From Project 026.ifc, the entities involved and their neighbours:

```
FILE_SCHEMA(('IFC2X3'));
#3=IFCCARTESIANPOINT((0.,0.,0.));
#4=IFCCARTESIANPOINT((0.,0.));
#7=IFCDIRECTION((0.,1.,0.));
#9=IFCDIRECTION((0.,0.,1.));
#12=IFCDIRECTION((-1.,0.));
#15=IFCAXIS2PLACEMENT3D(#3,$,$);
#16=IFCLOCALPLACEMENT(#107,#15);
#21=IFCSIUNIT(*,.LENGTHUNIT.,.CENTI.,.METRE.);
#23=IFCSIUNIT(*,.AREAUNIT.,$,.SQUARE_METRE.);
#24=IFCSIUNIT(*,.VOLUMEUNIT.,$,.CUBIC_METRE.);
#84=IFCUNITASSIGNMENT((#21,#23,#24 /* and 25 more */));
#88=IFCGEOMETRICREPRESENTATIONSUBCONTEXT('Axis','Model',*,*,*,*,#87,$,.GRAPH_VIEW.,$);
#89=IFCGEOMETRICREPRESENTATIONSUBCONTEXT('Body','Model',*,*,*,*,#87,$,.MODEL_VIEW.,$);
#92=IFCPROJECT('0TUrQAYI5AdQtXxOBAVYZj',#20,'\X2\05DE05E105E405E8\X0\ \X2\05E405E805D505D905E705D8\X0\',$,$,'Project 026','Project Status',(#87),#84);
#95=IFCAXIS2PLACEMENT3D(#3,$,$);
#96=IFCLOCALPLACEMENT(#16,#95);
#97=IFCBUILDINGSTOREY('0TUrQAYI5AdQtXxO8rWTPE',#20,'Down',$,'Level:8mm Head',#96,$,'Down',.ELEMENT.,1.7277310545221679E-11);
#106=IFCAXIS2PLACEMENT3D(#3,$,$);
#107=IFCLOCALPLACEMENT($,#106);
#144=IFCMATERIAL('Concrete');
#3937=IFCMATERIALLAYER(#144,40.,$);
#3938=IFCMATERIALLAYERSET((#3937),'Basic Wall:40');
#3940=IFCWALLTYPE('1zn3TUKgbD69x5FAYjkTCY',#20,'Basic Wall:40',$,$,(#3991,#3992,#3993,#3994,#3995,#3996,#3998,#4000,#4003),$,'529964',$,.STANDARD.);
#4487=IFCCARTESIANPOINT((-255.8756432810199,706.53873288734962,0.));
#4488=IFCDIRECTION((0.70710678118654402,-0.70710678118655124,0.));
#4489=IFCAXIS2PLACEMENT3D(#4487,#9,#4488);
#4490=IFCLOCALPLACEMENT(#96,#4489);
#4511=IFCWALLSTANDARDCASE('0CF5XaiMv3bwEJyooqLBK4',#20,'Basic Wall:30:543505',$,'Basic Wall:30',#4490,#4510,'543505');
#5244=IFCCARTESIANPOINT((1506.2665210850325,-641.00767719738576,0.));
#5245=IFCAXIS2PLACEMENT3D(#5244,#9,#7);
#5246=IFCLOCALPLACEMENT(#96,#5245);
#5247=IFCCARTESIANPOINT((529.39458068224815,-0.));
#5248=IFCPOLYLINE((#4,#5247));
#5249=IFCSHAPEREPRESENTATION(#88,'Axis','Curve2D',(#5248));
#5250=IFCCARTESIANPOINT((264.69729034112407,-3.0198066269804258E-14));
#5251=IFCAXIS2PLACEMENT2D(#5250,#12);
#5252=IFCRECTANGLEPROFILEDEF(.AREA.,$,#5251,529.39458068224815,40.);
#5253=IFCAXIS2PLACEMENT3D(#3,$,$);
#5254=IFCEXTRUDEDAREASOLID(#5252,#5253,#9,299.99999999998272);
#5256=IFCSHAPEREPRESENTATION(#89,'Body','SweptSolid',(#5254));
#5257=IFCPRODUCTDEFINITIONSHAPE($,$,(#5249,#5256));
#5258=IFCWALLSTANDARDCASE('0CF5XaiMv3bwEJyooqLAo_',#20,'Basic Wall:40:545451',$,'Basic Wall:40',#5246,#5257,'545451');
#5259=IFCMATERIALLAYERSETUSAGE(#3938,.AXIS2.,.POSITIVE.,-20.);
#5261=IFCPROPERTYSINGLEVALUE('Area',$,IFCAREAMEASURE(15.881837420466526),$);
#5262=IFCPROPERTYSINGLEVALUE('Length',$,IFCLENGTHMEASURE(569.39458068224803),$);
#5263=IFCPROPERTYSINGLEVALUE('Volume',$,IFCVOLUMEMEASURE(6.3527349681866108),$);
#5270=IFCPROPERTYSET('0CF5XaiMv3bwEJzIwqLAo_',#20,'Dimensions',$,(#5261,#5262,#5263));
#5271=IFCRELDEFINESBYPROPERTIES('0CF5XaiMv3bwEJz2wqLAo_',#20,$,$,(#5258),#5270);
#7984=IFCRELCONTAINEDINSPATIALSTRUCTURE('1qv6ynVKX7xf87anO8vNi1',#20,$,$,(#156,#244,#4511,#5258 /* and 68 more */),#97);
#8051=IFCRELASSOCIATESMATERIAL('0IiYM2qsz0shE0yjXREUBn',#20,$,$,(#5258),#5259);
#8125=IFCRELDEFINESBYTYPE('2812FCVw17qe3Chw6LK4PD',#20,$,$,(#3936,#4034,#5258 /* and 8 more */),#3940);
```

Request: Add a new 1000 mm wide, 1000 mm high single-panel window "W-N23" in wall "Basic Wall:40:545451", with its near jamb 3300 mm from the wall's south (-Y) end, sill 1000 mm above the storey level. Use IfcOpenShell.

```python
import numpy as np
import ifcopenshell
import ifcopenshell.api.feature
import ifcopenshell.api.geometry
import ifcopenshell.api.pset
import ifcopenshell.api.root
import ifcopenshell.api.spatial
import ifcopenshell.api.type
import ifcopenshell.geom
import ifcopenshell.util.element
import ifcopenshell.util.placement
import ifcopenshell.util.representation
import ifcopenshell.util.shape
import ifcopenshell.util.unit

model = ifcopenshell.open("Project 026.ifc")
unit_scale = ifcopenshell.util.unit.calculate_unit_scale(model)
area_scale = ifcopenshell.util.unit.calculate_unit_scale(model, "AREAUNIT")
volume_scale = ifcopenshell.util.unit.calculate_unit_scale(model, "VOLUMEUNIT")
settings = ifcopenshell.geom.settings()


def volume(element):
    """Net volume in cubic metres, openings subtracted."""
    shape = ifcopenshell.geom.create_shape(settings, element)
    return ifcopenshell.util.shape.get_volume(shape.geometry)


wall = model.by_guid("0CF5XaiMv3bwEJyooqLAo_")
storey = ifcopenshell.util.element.get_container(wall, ifc_class="IfcBuildingStorey")
context = ifcopenshell.util.representation.get_context(model, "Model", "Body", "MODEL_VIEW")
before = volume(wall)

width, height, from_end, sill = 1, 1, 3.3, 1  # metres

# The wall runs along its own X axis, and the end named is its -X end.
wall_shape = ifcopenshell.geom.create_shape(settings, wall)
x, y, z = ifcopenshell.util.shape.get_vertices(wall_shape.geometry).T
start = x.min() + from_end
face, thickness = float(y.min()), float(y.max() - y.min())
wall_matrix = ifcopenshell.util.placement.get_local_placement(wall.ObjectPlacement)
level = ifcopenshell.util.placement.get_local_placement(storey.ObjectPlacement)[2, 3]


def in_wall(x, y):
    """Placement at x, y metres in the wall's axes, at sill height."""
    matrix = wall_matrix.copy()
    matrix[:, 3] = wall_matrix @ np.array([x / unit_scale, y / unit_scale, 0.0, 1.0])
    matrix[2, 3] = level + sill / unit_scale
    return matrix


# Opening: a box that overshoots both wall faces by 50 mm.
opening = ifcopenshell.api.root.create_entity(model, ifc_class="IfcOpeningElement")
box = ifcopenshell.api.geometry.add_wall_representation(
    model, context=context, length=width, height=height, thickness=thickness + 0.1
)
ifcopenshell.api.geometry.assign_representation(model, product=opening, representation=box)
ifcopenshell.api.geometry.edit_object_placement(model, product=opening, matrix=in_wall(start, face - 0.05), is_si=False)
ifcopenshell.api.feature.add_feature(model, feature=opening, element=wall)

window = ifcopenshell.api.root.create_entity(model, ifc_class="IfcWindow", name="W-N23")
window.OverallWidth, window.OverallHeight = width / unit_scale, height / unit_scale
body = ifcopenshell.api.geometry.add_window_representation(
    model,
    context=context,
    overall_width=window.OverallWidth,
    overall_height=window.OverallHeight,
    partition_type="SINGLE_PANEL",
)
ifcopenshell.api.geometry.assign_representation(model, product=window, representation=body)
ifcopenshell.api.spatial.assign_container(model, products=[window], relating_structure=storey)
fills = ifcopenshell.api.feature.add_filling(model, opening=opening, element=window)
fills.OwnerHistory = window.OwnerHistory  # required in IFC2X3

# IFC2X3 keeps the operation on the window style.
style = ifcopenshell.api.root.create_entity(model, ifc_class="IfcWindowStyle", name="W-N23")
style.OperationType, style.ConstructionType = "SINGLE_PANEL", "NOTDEFINED"
style.ParameterTakesPrecedence = style.Sizeable = False
ifcopenshell.api.type.assign_type(model, related_objects=[window], relating_type=style)

# Centre the window in the wall's thickness.
ifcopenshell.api.geometry.edit_object_placement(model, product=window, matrix=in_wall(start, face), is_si=False)
window_shape = ifcopenshell.geom.create_shape(settings, window)
depth = ifcopenshell.util.shape.get_vertices(window_shape.geometry)[:, 1]
offset = face + thickness / 2 - (depth.min() + depth.max()) / 2
ifcopenshell.api.geometry.edit_object_placement(model, product=window, matrix=in_wall(start, offset), is_si=False)

after = volume(wall)

# Update the wall's stored quantities.
pset = model.by_id(ifcopenshell.util.element.get_pset(wall, "Dimensions", should_inherit=False)["id"])
ifcopenshell.api.pset.edit_pset(model, pset=pset, properties={
    "Area": model.create_entity("IfcAreaMeasure", after / thickness / area_scale),
    "Volume": model.create_entity("IfcVolumeMeasure", after / volume_scale),
})

print(f"wall volume {before:.3f} -> {after:.3f} m3")

model.write("Project 026_edited.ifc")
```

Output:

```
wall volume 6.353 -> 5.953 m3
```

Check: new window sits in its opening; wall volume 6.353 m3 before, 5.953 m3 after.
